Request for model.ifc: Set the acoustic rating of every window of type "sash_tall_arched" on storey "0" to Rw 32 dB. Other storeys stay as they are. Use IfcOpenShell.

First a look at what the model holds.

```python
import ifcopenshell
import ifcopenshell.util.element

model = ifcopenshell.open("model.ifc")
print(model.schema)
storey = next(s for s in model.by_type("IfcBuildingStorey") if s.Name == "0")
windows = [e for e in ifcopenshell.util.element.get_decomposition(storey) if e.is_a("IfcWindow")]
seen = {}
for e in windows:
    element_type = ifcopenshell.util.element.get_type(e)
    key = (element_type.Name if element_type != e and element_type else None, ifcopenshell.util.element.get_pset(e, "Pset_WindowCommon", "AcousticRating"))
    seen[key] = seen.get(key, 0) + 1
for (name, value), count in sorted(seen.items(), key=str):
    print(count, "x", name, "|", value)
```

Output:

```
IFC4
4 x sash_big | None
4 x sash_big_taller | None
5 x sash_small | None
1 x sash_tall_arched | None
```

```python
import ifcopenshell
import ifcopenshell.api.pset
import ifcopenshell.util.element

model = ifcopenshell.open("model.ifc")

storey = next(s for s in model.by_type("IfcBuildingStorey") if s.Name == "0")
windows = [e for e in ifcopenshell.util.element.get_decomposition(storey) if e.is_a("IfcWindow")]

count = 0
for e in windows:
    element_type = ifcopenshell.util.element.get_type(e)
    if element_type in (None, e) or element_type.Name != "sash_tall_arched":
        continue
    # add_pset returns the element's existing set when there is one.
    pset = ifcopenshell.api.pset.add_pset(model, product=e, name="Pset_WindowCommon")
    ifcopenshell.api.pset.edit_pset(model, pset=pset, properties={"AcousticRating": "Rw 32 dB"})
    count += 1

print(count, "windows updated")

model.write("model_rev.ifc")
```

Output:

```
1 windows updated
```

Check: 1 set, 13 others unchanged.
